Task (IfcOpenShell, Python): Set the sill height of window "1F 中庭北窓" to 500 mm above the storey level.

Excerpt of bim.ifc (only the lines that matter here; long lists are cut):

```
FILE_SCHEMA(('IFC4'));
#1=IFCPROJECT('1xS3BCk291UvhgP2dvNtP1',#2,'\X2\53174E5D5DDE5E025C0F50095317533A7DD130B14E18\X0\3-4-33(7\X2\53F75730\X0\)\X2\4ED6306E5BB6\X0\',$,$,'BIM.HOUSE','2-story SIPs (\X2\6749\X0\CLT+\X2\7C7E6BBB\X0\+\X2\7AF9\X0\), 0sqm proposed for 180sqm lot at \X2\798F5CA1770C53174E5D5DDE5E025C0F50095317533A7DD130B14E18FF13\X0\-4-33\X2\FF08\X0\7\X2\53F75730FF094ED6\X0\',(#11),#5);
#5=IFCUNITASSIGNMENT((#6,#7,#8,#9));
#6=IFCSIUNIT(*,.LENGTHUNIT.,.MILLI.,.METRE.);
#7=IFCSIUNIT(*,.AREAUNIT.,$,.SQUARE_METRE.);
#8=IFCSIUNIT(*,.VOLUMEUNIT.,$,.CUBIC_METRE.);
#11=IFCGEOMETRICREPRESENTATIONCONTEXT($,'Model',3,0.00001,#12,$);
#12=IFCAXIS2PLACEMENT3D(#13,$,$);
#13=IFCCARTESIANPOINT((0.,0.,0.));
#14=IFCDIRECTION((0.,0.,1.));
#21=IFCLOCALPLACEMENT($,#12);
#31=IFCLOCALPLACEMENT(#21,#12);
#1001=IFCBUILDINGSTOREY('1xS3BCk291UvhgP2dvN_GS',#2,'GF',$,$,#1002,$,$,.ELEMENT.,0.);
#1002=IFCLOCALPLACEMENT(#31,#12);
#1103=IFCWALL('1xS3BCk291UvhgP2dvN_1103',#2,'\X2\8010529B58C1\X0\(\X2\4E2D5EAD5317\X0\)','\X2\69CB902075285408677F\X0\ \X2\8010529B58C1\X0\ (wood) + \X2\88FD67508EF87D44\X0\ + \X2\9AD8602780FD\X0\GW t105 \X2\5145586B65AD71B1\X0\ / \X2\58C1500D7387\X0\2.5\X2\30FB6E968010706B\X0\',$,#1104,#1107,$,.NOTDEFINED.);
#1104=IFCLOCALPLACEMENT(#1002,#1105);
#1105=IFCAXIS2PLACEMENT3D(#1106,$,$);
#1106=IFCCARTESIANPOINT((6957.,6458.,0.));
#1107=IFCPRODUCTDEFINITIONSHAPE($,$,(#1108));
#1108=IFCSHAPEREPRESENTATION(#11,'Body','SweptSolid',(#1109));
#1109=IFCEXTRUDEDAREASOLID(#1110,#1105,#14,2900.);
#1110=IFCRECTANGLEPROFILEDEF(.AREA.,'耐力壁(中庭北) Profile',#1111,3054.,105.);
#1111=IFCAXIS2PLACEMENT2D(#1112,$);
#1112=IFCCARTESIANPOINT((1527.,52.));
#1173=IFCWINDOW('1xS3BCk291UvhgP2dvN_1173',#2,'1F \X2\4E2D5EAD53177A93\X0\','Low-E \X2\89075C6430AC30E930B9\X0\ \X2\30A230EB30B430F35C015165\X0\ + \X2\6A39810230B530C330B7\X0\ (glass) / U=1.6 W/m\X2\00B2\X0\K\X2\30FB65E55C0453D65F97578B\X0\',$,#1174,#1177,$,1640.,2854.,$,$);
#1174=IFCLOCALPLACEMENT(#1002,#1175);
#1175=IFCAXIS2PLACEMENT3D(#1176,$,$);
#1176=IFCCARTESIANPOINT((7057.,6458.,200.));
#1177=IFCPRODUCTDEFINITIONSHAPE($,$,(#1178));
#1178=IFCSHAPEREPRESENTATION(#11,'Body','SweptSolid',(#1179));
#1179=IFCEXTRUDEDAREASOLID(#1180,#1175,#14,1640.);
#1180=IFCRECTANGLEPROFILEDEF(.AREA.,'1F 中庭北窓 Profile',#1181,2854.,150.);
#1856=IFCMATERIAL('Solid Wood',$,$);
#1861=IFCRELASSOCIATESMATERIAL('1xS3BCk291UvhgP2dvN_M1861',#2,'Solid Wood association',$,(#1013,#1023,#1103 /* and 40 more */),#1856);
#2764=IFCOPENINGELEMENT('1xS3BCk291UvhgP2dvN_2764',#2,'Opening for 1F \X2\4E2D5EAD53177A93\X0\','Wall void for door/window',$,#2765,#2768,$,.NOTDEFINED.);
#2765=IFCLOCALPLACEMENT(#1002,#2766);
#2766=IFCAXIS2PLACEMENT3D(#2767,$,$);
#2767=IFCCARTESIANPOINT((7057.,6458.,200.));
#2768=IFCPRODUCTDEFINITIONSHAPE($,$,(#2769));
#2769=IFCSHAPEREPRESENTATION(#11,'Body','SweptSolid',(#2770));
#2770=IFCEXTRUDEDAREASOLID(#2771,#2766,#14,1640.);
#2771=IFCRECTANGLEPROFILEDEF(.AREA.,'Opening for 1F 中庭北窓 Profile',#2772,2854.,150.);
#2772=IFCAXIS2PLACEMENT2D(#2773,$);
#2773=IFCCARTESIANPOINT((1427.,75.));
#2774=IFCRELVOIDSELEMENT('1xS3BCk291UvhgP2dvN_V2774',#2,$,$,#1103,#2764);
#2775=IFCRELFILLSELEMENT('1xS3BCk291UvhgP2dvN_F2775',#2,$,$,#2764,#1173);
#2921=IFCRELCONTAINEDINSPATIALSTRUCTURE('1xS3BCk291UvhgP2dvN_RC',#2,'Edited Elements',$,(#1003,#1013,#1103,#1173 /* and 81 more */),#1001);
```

```python
import numpy as np
import ifcopenshell
import ifcopenshell.api.geometry
import ifcopenshell.geom
import ifcopenshell.util.element
import ifcopenshell.util.placement
import ifcopenshell.util.shape
import ifcopenshell.util.unit

model = ifcopenshell.open("bim.ifc")
unit_scale = ifcopenshell.util.unit.calculate_unit_scale(model)

window = model.by_guid("1xS3BCk291UvhgP2dvN_1173")
opening = window.FillsVoids[0].RelatingOpeningElement
storey = ifcopenshell.util.element.get_container(window, ifc_class="IfcBuildingStorey")
level = ifcopenshell.util.placement.get_local_placement(storey.ObjectPlacement)[2, 3]

# The opening's origin need not be at the sill, so measure its lowest point.
shape = ifcopenshell.geom.create_shape(ifcopenshell.geom.settings(), opening)
bottom = ifcopenshell.util.shape.get_shape_bottom_elevation(shape, shape.geometry) / unit_scale
dz = level + 0.5 / unit_scale - bottom

shift = np.array([0.0, 0.0, dz])
# The window is not placed relative to its opening, so move both.
for product in (opening, window):
    matrix = ifcopenshell.util.placement.get_local_placement(product.ObjectPlacement)
    matrix[:3, 3] += shift
    ifcopenshell.api.geometry.edit_object_placement(model, product=product, matrix=matrix, is_si=False)

print(f"moved by {dz * unit_scale:+.3f} m")

model.write("bim_updated.ifc")
```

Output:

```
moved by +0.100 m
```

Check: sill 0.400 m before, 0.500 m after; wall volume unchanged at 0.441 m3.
